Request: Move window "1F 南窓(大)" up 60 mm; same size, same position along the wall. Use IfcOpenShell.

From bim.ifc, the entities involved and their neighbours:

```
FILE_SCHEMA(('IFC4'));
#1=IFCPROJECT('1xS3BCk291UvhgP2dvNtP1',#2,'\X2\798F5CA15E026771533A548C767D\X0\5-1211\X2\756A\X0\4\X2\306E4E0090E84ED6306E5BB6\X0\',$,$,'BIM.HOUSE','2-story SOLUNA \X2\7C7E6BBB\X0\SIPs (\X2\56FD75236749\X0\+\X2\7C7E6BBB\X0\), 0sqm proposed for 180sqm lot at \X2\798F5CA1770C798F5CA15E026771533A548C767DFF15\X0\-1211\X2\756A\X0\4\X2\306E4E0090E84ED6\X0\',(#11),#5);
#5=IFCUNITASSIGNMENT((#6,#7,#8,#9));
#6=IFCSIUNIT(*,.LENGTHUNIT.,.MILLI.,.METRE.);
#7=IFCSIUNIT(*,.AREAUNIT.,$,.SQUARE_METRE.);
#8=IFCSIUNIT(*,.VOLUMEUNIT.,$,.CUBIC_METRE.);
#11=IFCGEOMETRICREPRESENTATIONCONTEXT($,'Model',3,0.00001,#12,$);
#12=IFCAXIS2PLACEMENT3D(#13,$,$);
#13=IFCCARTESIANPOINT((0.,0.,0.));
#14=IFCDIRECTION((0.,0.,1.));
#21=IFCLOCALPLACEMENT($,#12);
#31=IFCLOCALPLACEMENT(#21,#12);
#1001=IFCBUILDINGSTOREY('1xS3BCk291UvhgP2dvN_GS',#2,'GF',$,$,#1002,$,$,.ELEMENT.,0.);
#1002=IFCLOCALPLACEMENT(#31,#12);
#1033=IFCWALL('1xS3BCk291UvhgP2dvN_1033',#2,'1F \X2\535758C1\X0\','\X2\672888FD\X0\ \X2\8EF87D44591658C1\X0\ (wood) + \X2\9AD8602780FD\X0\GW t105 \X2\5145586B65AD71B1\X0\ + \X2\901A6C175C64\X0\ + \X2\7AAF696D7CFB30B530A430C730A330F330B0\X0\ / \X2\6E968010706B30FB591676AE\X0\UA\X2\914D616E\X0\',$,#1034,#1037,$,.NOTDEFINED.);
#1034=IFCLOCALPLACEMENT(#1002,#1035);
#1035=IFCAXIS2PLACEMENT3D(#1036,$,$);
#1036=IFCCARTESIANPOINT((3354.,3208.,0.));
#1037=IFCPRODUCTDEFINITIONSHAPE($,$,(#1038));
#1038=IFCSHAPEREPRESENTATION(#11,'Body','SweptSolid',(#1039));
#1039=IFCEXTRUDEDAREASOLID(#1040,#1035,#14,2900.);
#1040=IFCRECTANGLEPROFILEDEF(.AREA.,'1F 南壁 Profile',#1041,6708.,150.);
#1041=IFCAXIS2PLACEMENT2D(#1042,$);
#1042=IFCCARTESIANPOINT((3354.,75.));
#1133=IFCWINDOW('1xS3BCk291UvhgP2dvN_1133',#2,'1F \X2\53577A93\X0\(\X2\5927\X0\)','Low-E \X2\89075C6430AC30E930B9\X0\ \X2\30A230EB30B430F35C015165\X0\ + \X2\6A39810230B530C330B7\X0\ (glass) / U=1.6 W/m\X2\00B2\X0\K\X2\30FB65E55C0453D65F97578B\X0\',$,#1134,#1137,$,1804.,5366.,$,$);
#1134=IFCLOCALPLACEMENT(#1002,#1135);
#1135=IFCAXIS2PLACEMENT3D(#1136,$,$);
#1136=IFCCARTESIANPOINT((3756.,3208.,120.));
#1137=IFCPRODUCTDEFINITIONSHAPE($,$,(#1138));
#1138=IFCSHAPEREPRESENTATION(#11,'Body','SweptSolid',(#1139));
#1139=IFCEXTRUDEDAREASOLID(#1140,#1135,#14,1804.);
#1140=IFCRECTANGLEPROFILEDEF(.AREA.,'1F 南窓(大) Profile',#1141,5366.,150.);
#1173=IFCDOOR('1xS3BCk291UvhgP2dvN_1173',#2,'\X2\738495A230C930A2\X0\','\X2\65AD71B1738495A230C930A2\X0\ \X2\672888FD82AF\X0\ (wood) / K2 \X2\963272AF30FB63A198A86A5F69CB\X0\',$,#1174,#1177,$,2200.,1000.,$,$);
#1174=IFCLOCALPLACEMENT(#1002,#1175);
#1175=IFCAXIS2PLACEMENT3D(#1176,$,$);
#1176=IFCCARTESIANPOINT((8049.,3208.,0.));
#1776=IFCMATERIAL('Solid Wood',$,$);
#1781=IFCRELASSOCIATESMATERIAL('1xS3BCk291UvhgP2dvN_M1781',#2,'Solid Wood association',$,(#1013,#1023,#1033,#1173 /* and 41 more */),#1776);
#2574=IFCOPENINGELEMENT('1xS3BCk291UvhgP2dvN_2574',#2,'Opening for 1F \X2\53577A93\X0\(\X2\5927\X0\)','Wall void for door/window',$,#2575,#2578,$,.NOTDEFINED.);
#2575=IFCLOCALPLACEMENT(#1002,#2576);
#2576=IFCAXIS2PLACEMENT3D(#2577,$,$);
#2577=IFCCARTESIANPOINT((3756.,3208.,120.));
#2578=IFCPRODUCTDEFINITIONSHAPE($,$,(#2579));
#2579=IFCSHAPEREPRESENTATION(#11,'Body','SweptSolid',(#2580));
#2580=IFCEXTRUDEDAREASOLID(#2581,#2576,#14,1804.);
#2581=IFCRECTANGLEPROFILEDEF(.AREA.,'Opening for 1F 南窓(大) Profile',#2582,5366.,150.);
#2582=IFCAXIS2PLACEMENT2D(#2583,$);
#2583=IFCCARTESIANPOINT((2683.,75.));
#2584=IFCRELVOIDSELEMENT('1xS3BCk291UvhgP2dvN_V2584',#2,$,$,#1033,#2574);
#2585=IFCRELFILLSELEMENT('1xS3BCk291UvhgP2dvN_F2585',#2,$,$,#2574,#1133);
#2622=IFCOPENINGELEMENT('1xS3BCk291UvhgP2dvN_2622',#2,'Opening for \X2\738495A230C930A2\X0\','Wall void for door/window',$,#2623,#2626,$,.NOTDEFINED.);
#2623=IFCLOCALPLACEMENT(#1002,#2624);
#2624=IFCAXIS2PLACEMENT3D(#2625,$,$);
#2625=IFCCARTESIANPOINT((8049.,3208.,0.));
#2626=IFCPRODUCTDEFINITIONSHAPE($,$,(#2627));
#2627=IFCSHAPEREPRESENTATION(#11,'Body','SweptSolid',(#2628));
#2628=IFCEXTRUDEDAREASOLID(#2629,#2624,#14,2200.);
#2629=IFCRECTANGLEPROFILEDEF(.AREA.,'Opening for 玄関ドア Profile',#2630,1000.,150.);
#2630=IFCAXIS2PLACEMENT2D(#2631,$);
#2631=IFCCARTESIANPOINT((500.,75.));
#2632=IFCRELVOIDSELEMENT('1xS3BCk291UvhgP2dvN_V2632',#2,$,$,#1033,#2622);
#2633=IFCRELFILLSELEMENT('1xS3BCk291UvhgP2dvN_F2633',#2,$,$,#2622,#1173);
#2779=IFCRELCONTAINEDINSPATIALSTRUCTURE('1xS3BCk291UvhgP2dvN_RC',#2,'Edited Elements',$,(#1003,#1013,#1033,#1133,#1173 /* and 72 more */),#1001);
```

```python
import numpy as np
import ifcopenshell
import ifcopenshell.api.geometry
import ifcopenshell.util.placement
import ifcopenshell.util.unit

model = ifcopenshell.open("bim.ifc")
unit_scale = ifcopenshell.util.unit.calculate_unit_scale(model)

window = model.by_id(1133)
opening = window.FillsVoids[0].RelatingOpeningElement
dz = 0.06 / unit_scale

shift = np.array([0.0, 0.0, dz])
# The window is not placed relative to its opening, so move both.
for product in (opening, window):
    matrix = ifcopenshell.util.placement.get_local_placement(product.ObjectPlacement)
    matrix[:3, 3] += shift
    ifcopenshell.api.geometry.edit_object_placement(model, product=product, matrix=matrix, is_si=False)

print(f"moved by {dz * unit_scale:+.3f} m")

model.write("bim_rev.ifc")
```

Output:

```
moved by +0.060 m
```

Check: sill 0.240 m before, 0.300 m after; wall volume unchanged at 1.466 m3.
